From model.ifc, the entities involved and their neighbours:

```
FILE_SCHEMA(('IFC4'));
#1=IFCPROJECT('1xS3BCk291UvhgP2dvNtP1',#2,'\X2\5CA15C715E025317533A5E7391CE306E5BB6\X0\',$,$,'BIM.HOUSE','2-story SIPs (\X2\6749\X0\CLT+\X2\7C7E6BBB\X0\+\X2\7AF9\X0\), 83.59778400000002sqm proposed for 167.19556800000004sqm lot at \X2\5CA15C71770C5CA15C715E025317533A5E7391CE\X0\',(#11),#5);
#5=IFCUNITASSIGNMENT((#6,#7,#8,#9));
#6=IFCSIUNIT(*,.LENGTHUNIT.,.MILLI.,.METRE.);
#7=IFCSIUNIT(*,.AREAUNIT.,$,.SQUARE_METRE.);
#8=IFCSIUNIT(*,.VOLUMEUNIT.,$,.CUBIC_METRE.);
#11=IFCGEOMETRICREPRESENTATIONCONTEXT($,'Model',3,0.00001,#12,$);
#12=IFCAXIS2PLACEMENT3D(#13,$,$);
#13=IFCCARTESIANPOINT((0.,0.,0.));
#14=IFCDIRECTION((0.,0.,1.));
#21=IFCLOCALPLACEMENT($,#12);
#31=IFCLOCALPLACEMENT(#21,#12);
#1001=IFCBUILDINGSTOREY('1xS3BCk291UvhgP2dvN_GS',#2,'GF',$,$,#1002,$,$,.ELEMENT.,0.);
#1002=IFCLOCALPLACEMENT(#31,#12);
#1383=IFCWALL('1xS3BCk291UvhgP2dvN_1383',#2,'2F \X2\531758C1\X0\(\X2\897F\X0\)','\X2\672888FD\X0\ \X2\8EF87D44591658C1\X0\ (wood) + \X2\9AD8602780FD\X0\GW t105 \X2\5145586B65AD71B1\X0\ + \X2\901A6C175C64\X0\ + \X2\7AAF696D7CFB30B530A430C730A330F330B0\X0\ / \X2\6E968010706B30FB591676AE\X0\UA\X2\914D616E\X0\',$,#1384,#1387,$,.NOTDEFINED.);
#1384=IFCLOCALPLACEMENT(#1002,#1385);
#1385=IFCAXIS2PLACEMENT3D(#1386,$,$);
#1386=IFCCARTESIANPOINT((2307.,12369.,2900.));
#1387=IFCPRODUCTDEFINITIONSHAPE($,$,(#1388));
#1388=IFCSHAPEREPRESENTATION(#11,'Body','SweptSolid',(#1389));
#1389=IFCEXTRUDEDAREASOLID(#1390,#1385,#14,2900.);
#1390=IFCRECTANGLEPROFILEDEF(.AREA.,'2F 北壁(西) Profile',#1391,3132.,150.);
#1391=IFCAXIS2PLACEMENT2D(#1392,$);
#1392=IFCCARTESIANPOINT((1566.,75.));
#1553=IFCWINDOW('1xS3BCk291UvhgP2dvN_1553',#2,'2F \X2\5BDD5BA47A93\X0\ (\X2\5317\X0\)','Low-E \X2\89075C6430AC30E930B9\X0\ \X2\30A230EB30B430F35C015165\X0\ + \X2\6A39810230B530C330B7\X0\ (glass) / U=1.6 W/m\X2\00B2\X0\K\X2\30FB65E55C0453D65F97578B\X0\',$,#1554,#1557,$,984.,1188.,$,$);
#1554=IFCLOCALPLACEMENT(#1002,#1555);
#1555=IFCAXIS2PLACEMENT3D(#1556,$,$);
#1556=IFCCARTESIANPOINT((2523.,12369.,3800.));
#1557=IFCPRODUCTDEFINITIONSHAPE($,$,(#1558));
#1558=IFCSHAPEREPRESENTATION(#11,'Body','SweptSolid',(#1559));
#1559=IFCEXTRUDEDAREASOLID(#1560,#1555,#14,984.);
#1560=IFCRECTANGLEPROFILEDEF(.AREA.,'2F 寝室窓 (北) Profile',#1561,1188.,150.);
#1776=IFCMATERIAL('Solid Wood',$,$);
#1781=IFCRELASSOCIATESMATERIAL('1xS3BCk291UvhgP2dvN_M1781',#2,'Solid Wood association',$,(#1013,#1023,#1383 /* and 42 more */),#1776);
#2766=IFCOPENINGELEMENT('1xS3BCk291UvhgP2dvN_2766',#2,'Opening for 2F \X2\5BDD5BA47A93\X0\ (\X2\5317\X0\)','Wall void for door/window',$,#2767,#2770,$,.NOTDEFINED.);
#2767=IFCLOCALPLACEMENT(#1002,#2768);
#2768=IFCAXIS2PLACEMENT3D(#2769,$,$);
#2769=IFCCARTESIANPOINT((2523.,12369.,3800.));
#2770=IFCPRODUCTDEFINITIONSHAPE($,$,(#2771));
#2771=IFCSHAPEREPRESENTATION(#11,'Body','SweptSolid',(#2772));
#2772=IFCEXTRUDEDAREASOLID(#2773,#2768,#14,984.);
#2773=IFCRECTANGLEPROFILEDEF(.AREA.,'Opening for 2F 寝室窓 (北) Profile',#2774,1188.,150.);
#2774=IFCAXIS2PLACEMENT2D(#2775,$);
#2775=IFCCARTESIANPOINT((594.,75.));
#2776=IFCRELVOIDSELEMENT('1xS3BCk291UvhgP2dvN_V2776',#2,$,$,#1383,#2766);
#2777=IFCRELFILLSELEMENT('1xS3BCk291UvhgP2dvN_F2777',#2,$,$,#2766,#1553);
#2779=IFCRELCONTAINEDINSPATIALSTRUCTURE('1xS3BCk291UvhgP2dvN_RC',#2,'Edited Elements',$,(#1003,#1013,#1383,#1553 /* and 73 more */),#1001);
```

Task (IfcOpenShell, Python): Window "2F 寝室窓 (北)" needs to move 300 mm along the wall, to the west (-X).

```python
import ifcopenshell
import ifcopenshell.api.geometry
import ifcopenshell.util.placement

model = ifcopenshell.open("model.ifc")

window = model.by_guid("1xS3BCk291UvhgP2dvN_1553")
opening = window.FillsVoids[0].RelatingOpeningElement
wall = opening.VoidsElements[0].RelatingBuildingElement

wall_matrix = ifcopenshell.util.placement.get_local_placement(wall.ObjectPlacement)
shift = wall_matrix[:3, 0] * -300.0
before = ifcopenshell.util.placement.get_local_placement(window.ObjectPlacement)[:3, 3].copy()

# The window is not placed relative to its opening, so move both.
for product in (opening, window):
    matrix = ifcopenshell.util.placement.get_local_placement(product.ObjectPlacement)
    matrix[:3, 3] += shift
    ifcopenshell.api.geometry.edit_object_placement(model, product=product, matrix=matrix, is_si=False)

after = ifcopenshell.util.placement.get_local_placement(window.ObjectPlacement)[:3, 3]
print("window moved by", (after - before).round(3) + 0.0)

model.write("model_updated.ifc")
```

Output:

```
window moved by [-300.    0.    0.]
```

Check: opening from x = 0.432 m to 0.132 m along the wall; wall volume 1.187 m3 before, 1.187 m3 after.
